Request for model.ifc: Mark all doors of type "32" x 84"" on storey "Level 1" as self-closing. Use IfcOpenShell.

First a look at what the model holds.

```python
import ifcopenshell
import ifcopenshell.util.element

model = ifcopenshell.open("model.ifc")
print(model.schema)
storey = next(s for s in model.by_type("IfcBuildingStorey") if s.Name == "Level 1")
doors = [e for e in ifcopenshell.util.element.get_decomposition(storey) if e.is_a("IfcDoor")]
seen = {}
for e in doors:
    element_type = ifcopenshell.util.element.get_type(e)
    key = (element_type.Name if element_type != e and element_type else None, ifcopenshell.util.element.get_pset(e, "Pset_DoorCommon", "SelfClosing"))
    seen[key] = seen.get(key, 0) + 1
for (name, value), count in sorted(seen.items(), key=str):
    print(count, "x", name, "|", value)
```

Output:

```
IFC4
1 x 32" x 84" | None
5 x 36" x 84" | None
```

```python
import ifcopenshell
import ifcopenshell.api.pset
import ifcopenshell.util.element

model = ifcopenshell.open("model.ifc")

storey = next(s for s in model.by_type("IfcBuildingStorey") if s.Name == "Level 1")
doors = [e for e in ifcopenshell.util.element.get_decomposition(storey) if e.is_a("IfcDoor")]

count = 0
for e in doors:
    element_type = ifcopenshell.util.element.get_type(e)
    if element_type in (None, e) or element_type.Name != '32" x 84"':
        continue
    # add_pset returns the element's existing set when there is one.
    pset = ifcopenshell.api.pset.add_pset(model, product=e, name="Pset_DoorCommon")
    ifcopenshell.api.pset.edit_pset(model, pset=pset, properties={"SelfClosing": True})
    count += 1

print(count, "doors updated")

model.write("model_v2.ifc")
```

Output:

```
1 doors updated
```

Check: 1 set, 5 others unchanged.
